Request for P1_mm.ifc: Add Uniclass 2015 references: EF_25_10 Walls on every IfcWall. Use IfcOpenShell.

First a look at what the model holds.

```python
import ifcopenshell

model = ifcopenshell.open("P1_mm.ifc")
print(model.schema)
print("classifications:", [c.Name for c in model.by_type("IfcClassification")])
for ifc_class in ("IfcDoor", "IfcRoof", "IfcStair", "IfcWall", "IfcWindow"):
    print(ifc_class, len(model.by_type(ifc_class)))
```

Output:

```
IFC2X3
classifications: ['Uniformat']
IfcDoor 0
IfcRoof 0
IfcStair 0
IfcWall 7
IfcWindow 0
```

```python
import ifcopenshell
import ifcopenshell.api.classification

model = ifcopenshell.open("P1_mm.ifc")

# IFC2X3 requires Source and Edition and has no link from the project to the system.
system = model.create_entity("IfcClassification", Source="NBS", Edition="2015", Name="Uniclass 2015")

codes = {
    "IfcWall": ("EF_25_10", "Walls"),
}
for ifc_class, (code, name) in codes.items():
    products = model.by_type(ifc_class)
    ifcopenshell.api.classification.add_reference(
        model, products=products, classification=system, identification=code, name=name
    )
    print(code, len(products))

model.write("P1_mm_rev.ifc")
```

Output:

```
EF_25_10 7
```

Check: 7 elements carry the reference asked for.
